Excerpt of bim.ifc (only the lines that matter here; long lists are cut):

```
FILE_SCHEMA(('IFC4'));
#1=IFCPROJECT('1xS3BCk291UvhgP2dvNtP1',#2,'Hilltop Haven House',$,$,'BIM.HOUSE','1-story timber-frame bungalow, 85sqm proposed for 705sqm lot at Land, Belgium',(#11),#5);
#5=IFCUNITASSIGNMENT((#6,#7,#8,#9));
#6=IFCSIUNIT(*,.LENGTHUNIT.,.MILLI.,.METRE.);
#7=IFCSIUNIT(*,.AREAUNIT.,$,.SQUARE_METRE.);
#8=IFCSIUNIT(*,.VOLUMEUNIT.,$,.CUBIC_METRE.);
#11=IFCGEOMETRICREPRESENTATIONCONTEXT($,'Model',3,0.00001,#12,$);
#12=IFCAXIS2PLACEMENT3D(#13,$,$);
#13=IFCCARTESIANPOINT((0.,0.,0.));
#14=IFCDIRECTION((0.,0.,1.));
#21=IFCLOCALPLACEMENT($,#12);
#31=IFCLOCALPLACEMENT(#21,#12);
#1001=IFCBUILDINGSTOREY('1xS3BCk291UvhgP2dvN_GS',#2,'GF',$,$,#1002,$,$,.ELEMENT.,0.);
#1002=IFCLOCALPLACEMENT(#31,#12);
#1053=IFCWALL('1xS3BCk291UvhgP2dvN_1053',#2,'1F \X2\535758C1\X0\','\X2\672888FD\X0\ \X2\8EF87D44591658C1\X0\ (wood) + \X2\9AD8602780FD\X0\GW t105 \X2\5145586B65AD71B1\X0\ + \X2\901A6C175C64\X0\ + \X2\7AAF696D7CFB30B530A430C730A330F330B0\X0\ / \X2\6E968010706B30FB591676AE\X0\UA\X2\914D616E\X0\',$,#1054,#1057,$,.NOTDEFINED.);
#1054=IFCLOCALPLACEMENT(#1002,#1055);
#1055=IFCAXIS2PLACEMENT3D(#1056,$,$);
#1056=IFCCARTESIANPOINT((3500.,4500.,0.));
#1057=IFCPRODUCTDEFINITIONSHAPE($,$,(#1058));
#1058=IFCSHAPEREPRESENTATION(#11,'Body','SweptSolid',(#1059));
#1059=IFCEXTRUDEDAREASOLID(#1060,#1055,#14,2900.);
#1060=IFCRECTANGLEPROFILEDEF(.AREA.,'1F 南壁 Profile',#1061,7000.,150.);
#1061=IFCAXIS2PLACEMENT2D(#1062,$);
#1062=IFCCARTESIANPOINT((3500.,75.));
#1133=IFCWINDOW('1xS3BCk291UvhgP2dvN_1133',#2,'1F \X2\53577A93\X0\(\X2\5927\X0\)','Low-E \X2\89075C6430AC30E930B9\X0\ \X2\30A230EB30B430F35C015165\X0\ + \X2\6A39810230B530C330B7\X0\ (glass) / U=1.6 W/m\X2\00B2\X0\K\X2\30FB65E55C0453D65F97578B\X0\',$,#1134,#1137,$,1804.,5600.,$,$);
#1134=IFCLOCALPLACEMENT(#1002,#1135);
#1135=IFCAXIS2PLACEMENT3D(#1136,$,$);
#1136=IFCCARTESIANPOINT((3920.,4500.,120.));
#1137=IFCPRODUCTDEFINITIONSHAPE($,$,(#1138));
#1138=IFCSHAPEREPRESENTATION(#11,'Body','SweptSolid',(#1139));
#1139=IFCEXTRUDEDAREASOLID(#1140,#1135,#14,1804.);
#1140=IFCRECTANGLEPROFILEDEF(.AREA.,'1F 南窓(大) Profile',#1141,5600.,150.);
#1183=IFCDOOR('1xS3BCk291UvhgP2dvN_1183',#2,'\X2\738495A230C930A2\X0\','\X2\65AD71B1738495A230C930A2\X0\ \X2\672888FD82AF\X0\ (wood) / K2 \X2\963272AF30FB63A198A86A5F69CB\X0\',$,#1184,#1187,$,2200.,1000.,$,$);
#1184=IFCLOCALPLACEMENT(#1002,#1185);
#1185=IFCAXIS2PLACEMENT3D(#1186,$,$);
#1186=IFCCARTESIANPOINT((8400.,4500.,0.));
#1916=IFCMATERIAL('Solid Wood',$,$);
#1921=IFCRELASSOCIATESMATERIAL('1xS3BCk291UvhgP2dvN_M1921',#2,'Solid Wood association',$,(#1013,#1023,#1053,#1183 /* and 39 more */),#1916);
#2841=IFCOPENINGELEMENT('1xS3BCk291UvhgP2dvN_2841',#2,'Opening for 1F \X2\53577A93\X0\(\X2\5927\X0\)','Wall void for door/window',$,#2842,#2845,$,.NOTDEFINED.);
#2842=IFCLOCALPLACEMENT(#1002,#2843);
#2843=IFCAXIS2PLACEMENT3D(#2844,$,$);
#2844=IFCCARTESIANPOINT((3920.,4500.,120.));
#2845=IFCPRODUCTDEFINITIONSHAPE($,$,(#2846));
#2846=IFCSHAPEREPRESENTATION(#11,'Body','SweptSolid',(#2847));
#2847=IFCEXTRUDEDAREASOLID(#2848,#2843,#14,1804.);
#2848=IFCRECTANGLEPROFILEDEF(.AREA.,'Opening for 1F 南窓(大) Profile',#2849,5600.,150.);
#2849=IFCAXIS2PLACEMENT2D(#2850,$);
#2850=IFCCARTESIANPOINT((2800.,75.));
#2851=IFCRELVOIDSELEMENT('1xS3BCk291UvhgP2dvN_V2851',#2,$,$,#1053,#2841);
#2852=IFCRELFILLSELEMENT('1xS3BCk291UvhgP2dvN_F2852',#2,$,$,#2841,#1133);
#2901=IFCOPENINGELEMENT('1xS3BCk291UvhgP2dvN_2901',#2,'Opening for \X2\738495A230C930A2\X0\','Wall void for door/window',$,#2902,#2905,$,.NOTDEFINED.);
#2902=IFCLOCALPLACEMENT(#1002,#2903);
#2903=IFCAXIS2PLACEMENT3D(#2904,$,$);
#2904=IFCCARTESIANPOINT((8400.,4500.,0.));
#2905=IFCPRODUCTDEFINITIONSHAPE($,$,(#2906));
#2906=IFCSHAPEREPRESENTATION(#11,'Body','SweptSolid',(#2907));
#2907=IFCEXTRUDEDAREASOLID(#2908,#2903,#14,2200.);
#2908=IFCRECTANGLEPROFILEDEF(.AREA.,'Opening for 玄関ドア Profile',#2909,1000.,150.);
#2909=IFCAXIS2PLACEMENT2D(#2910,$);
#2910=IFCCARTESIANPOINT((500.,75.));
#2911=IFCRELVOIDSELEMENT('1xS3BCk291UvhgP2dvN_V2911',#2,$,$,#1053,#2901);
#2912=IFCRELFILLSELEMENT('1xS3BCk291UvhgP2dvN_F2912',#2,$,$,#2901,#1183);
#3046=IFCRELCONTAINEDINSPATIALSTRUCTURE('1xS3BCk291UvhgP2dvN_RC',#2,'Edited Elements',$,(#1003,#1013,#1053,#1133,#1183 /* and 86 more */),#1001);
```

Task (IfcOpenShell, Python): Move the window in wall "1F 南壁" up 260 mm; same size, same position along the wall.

```python
import numpy as np
import ifcopenshell
import ifcopenshell.api.geometry
import ifcopenshell.util.placement
import ifcopenshell.util.unit

model = ifcopenshell.open("bim.ifc")
unit_scale = ifcopenshell.util.unit.calculate_unit_scale(model)

window = model.by_id(1133)
opening = window.FillsVoids[0].RelatingOpeningElement
dz = 0.26 / unit_scale

shift = np.array([0.0, 0.0, dz])
# The window is not placed relative to its opening, so move both.
for product in (opening, window):
    matrix = ifcopenshell.util.placement.get_local_placement(product.ObjectPlacement)
    matrix[:3, 3] += shift
    ifcopenshell.api.geometry.edit_object_placement(model, product=product, matrix=matrix, is_si=False)

print(f"moved by {dz * unit_scale:+.3f} m")

model.write("bim-out.ifc")
```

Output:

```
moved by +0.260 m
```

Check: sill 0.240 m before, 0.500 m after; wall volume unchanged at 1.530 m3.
